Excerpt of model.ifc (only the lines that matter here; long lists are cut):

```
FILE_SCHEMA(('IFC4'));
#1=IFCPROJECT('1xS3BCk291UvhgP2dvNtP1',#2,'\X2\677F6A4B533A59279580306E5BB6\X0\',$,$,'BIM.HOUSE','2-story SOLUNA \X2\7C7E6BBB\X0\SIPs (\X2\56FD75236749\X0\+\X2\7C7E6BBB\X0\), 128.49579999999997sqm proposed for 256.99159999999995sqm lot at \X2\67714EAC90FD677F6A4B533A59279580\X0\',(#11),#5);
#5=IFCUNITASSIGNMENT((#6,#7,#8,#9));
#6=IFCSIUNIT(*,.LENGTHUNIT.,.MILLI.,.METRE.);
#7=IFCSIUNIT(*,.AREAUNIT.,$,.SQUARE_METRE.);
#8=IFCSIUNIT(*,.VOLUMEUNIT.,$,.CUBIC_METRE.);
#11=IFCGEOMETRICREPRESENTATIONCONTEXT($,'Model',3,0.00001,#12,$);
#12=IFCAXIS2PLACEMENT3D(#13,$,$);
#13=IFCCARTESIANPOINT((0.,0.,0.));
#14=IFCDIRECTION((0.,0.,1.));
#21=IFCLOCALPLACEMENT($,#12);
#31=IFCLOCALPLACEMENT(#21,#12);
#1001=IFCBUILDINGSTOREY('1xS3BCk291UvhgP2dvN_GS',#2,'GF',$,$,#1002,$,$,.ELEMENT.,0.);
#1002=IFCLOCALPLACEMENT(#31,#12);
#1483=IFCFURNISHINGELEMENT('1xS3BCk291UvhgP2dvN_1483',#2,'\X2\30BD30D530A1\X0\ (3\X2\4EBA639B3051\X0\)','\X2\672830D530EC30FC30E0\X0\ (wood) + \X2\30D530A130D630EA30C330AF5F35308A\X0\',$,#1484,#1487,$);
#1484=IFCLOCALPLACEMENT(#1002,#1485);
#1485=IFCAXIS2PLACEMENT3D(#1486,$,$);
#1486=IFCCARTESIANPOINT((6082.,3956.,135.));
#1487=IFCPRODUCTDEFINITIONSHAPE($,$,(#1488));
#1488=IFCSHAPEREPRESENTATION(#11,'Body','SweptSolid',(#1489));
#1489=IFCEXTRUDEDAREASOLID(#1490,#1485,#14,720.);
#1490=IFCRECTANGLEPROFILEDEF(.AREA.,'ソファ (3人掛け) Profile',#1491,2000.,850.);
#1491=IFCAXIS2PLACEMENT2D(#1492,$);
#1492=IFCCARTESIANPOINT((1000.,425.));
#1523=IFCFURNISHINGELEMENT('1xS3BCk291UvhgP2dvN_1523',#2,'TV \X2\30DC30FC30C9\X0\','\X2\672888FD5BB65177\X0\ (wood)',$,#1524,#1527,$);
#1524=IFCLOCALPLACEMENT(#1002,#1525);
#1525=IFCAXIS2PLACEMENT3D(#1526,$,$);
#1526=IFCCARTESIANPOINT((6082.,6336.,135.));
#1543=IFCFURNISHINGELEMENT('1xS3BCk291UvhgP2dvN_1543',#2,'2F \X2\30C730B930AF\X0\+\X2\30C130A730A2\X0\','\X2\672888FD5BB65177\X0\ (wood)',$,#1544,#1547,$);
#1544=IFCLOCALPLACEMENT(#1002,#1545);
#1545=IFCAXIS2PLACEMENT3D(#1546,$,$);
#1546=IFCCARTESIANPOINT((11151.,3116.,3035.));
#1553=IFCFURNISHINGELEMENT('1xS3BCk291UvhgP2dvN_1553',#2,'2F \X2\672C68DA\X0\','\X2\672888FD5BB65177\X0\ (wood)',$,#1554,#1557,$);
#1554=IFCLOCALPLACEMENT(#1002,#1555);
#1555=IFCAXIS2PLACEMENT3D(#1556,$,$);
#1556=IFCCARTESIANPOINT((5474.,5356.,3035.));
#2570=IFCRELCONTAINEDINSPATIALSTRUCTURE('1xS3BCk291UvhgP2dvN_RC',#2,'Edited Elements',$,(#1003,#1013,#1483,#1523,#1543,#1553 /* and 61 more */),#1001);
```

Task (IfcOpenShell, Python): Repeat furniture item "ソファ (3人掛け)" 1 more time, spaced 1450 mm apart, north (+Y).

```python
import numpy as np
import ifcopenshell
import ifcopenshell.api.geometry
import ifcopenshell.api.root
import ifcopenshell.util.element
import ifcopenshell.util.placement
import ifcopenshell.util.unit

model = ifcopenshell.open("model.ifc")
unit_scale = ifcopenshell.util.unit.calculate_unit_scale(model)


def reuse_history(source, copy):
    """copy_class also copies each property set's owner history, people and application; keep the originals."""
    for rel in copy.IsDefinedBy:
        if rel.is_a("IfcRelDefinesByProperties") and (history := rel.RelatingPropertyDefinition.OwnerHistory):
            rel.RelatingPropertyDefinition.OwnerHistory = source.OwnerHistory
            ifcopenshell.util.element.remove_deep2(model, history)


source = model.by_guid("1xS3BCk291UvhgP2dvN_1483")
base = ifcopenshell.util.placement.get_local_placement(source.ObjectPlacement)
step = np.array([0.0, 1.0, 0.0]) * 1.45 / unit_scale

for i in range(1, 2):
    copy = ifcopenshell.api.root.copy_class(model, product=source)
    copy.Representation = ifcopenshell.util.element.copy_deep(
        model, source.Representation, exclude=["IfcGeometricRepresentationContext", "IfcRepresentationMap"]
    )
    reuse_history(source, copy)
    matrix = base.copy()
    matrix[:3, 3] += i * step
    print("added at", matrix[:3, 3].round(3) + 0.0)
    ifcopenshell.api.geometry.edit_object_placement(model, product=copy, matrix=matrix, is_si=False)

model.write("model-out.ifc")
```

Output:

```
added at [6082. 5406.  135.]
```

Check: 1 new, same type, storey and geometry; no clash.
